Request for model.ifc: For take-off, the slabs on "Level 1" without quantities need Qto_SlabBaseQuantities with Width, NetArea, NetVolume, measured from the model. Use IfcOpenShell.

First a look at what the model holds.

```python
import ifcopenshell
import ifcopenshell.util.element
import ifcopenshell.util.unit

model = ifcopenshell.open("model.ifc")
print(model.schema)
for unit_type in ("LENGTHUNIT", "AREAUNIT", "VOLUMEUNIT"):
    print(unit_type, ifcopenshell.util.unit.calculate_unit_scale(model, unit_type))
storey = next(s for s in model.by_type("IfcBuildingStorey") if s.Name == "Level 1")
slabs = [e for e in ifcopenshell.util.element.get_decomposition(storey) if e.is_a("IfcSlab")]
for e in sorted(slabs, key=lambda e: e.id()):
    print(e.id(), e.is_a(), e.Name, list(ifcopenshell.util.element.get_psets(e, qtos_only=True)), sep=" | ")
```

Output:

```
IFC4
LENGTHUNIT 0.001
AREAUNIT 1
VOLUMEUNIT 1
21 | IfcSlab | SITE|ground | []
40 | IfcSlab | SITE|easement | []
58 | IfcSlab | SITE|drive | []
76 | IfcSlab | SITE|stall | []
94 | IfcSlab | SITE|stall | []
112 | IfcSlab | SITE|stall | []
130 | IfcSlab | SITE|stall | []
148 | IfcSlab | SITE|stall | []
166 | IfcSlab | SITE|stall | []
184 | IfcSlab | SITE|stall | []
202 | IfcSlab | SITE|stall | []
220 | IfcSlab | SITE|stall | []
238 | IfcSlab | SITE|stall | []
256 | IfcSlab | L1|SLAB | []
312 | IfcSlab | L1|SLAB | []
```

```python
import ifcopenshell
import ifcopenshell.api.pset
import ifcopenshell.geom
import ifcopenshell.util.element
import ifcopenshell.util.shape
import ifcopenshell.util.unit

model = ifcopenshell.open("model.ifc")
unit_scale = ifcopenshell.util.unit.calculate_unit_scale(model)
area_scale = ifcopenshell.util.unit.calculate_unit_scale(model, "AREAUNIT")
volume_scale = ifcopenshell.util.unit.calculate_unit_scale(model, "VOLUMEUNIT")
settings = ifcopenshell.geom.settings()

storey = next(s for s in model.by_type("IfcBuildingStorey") if s.Name == "Level 1")
slabs = [e for e in ifcopenshell.util.element.get_decomposition(storey) if e.is_a("IfcSlab")]

for e in sorted(slabs, key=lambda e: e.id()):
    if ifcopenshell.util.element.get_psets(e, qtos_only=True, should_inherit=False):
        continue
    # Geometry comes back in metres, in the element's own axes.
    shape = ifcopenshell.geom.create_shape(settings, e)
    values = {
        "Width": ifcopenshell.util.shape.get_z(shape.geometry) / unit_scale,
        "NetArea": ifcopenshell.util.shape.get_footprint_area(shape.geometry) / area_scale,
        "NetVolume": ifcopenshell.util.shape.get_volume(shape.geometry) / volume_scale,
    }
    qto = ifcopenshell.api.pset.add_qto(model, product=e, name="Qto_SlabBaseQuantities")
    ifcopenshell.api.pset.edit_qto(model, qto=qto, properties=values)
    print(e.id(), {k: round(v, 3) for k, v in values.items()})

model.write("model_v2.ifc")
```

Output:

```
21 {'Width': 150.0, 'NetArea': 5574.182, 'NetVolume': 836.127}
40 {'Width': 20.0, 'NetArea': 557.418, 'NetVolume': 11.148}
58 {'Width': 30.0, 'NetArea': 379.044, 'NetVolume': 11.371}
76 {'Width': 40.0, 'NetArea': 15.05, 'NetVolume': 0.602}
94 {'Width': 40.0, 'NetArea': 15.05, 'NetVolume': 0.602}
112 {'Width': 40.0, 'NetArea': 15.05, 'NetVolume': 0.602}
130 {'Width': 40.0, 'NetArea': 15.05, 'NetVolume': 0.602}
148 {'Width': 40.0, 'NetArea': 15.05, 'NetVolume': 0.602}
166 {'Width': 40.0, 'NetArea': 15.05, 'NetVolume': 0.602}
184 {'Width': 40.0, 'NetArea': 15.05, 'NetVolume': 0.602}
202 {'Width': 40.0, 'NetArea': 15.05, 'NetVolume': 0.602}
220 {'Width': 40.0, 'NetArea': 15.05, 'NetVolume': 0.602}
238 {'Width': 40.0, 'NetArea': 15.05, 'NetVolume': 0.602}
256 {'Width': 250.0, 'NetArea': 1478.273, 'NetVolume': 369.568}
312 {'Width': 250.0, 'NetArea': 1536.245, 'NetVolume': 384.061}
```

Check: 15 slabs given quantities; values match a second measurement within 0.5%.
